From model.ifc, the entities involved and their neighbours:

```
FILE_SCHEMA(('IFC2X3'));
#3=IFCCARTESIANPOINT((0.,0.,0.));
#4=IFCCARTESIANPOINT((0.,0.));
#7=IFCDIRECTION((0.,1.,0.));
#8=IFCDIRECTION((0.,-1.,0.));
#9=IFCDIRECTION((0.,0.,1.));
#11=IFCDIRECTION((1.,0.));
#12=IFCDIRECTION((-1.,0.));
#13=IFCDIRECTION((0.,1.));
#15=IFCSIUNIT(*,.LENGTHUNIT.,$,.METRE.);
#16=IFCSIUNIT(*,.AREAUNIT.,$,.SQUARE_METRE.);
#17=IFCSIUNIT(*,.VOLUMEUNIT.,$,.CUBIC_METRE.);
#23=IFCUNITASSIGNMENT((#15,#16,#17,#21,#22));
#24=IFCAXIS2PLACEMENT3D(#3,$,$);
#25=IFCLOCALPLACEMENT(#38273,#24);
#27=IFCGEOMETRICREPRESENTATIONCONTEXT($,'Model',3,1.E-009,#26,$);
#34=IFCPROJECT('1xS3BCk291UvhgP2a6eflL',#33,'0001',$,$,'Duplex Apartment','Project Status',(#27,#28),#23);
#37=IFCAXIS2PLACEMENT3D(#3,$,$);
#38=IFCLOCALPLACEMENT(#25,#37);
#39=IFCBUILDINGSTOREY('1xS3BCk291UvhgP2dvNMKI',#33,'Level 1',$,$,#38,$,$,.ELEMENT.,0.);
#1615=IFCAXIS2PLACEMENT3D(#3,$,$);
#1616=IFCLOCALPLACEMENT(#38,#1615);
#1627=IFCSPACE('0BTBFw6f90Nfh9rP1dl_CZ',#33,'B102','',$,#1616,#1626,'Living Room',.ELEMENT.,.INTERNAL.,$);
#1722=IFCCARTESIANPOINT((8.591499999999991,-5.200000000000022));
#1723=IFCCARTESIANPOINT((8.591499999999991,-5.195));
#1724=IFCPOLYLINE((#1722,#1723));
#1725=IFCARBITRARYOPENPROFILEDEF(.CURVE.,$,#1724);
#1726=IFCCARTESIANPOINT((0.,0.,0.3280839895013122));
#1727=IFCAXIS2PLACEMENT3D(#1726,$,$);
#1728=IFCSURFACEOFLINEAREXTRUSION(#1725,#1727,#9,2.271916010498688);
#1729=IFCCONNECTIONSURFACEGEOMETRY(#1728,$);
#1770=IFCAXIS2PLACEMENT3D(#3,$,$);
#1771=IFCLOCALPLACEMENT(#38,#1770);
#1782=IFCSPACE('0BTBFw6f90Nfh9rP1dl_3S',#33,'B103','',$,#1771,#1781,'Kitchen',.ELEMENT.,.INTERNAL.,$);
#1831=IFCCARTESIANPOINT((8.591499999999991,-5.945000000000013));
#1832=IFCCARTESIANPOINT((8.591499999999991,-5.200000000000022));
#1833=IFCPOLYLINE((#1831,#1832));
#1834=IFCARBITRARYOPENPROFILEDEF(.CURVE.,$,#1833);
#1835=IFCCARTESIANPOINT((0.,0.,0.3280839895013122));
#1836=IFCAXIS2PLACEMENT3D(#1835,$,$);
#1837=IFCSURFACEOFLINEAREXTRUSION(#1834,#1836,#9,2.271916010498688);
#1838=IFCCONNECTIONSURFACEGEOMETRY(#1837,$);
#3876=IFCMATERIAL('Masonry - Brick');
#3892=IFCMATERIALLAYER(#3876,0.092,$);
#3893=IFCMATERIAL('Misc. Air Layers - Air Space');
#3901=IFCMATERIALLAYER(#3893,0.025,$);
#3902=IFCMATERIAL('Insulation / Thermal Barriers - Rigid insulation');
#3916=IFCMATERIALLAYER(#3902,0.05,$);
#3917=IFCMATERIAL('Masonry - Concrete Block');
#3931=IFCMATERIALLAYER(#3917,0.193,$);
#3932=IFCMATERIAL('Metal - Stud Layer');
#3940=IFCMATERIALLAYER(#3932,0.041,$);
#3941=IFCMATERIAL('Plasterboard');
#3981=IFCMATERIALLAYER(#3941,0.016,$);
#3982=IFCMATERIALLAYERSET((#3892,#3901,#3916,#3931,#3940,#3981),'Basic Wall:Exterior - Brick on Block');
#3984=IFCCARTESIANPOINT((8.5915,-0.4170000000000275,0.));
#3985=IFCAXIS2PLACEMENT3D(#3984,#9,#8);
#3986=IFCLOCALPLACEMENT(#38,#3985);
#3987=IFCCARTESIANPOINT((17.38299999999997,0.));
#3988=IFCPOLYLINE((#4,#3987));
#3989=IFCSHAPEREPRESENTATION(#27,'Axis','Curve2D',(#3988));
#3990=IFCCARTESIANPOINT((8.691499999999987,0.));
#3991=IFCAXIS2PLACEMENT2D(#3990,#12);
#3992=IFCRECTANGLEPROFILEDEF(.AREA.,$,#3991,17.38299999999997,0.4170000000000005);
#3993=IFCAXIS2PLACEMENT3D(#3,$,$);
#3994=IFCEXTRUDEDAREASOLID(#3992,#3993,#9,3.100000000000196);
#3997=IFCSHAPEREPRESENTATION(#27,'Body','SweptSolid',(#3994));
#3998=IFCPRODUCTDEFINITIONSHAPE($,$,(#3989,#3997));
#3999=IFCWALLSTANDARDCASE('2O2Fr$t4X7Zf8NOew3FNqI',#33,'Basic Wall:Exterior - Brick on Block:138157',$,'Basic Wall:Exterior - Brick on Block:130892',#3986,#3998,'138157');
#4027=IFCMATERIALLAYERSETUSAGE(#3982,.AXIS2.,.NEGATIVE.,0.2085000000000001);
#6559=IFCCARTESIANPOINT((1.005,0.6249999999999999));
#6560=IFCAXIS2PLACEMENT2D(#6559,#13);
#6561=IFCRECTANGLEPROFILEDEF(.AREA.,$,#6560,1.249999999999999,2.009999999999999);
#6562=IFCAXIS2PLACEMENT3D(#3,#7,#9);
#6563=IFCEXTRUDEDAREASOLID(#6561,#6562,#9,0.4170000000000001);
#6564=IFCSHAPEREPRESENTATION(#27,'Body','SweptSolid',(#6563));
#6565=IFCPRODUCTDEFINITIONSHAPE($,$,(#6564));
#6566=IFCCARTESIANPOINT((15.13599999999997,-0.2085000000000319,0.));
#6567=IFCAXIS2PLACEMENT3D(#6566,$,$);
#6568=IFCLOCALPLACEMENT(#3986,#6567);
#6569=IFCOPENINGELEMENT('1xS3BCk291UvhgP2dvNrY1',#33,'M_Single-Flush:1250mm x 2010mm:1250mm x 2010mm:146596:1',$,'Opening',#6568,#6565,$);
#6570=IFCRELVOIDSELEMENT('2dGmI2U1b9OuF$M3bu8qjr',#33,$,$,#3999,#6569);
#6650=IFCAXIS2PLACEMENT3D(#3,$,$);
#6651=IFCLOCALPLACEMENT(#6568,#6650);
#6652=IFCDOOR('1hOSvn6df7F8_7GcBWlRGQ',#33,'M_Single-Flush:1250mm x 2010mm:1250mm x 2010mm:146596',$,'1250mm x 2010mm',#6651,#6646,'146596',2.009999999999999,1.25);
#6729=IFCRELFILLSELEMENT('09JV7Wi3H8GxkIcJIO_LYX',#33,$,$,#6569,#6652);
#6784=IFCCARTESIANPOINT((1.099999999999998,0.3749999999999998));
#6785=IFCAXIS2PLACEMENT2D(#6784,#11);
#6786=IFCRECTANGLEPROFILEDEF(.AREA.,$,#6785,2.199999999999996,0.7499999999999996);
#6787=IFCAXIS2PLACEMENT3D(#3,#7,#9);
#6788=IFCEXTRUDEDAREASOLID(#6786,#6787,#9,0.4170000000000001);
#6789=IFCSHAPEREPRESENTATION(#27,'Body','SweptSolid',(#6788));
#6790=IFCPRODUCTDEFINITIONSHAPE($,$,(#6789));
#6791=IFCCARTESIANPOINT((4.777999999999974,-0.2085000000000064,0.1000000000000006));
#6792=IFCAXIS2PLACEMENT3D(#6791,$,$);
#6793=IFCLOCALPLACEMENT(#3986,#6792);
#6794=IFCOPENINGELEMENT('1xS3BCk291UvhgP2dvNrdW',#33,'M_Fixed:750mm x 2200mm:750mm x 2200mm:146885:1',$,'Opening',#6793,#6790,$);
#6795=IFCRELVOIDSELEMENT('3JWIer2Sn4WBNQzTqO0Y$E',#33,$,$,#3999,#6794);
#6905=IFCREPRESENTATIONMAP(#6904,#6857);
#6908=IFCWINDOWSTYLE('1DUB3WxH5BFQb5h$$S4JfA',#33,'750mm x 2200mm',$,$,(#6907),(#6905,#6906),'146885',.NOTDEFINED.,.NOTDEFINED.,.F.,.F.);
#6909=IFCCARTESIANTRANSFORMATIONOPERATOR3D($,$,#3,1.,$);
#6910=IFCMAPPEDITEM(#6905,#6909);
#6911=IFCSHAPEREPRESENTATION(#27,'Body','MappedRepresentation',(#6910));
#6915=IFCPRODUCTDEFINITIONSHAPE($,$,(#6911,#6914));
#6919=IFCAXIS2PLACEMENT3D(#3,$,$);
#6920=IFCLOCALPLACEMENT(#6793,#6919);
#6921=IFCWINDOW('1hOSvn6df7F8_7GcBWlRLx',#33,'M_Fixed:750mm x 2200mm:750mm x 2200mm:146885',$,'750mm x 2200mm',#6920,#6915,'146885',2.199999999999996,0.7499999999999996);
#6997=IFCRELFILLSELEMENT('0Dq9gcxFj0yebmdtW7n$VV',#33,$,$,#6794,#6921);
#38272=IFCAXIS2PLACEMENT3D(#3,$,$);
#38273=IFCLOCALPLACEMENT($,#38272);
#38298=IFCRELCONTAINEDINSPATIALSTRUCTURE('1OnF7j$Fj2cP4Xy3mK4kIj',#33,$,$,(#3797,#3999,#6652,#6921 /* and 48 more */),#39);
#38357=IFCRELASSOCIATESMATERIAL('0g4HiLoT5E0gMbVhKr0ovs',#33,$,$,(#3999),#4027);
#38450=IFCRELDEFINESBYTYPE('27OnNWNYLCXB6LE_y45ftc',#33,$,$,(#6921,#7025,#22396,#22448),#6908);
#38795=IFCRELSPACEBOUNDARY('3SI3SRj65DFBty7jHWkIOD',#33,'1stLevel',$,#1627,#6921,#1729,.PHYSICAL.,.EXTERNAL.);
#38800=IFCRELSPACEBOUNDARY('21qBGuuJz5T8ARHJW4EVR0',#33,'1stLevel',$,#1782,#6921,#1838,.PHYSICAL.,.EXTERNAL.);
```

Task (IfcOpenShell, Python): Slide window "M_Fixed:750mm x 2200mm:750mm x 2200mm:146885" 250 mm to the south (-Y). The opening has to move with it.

```python
import numpy as np
import ifcopenshell
import ifcopenshell.api.geometry
import ifcopenshell.util.placement
import ifcopenshell.util.unit

model = ifcopenshell.open("model.ifc")
unit_scale = ifcopenshell.util.unit.calculate_unit_scale(model)

window = model.by_id(6921)
opening = window.FillsVoids[0].RelatingOpeningElement
wall = opening.VoidsElements[0].RelatingBuildingElement

wall_matrix = ifcopenshell.util.placement.get_local_placement(wall.ObjectPlacement)
shift = wall_matrix[:3, 0] * 0.25 / unit_scale
before = ifcopenshell.util.placement.get_local_placement(window.ObjectPlacement)[:3, 3].copy()

# The window is placed relative to its opening, so it follows when the opening moves.
matrix = ifcopenshell.util.placement.get_local_placement(opening.ObjectPlacement)
matrix[:3, 3] += shift
ifcopenshell.api.geometry.edit_object_placement(
    model, product=opening, matrix=matrix, is_si=False, should_transform_children=True
)

# Space boundary surfaces are stored in each space's coordinates; move them too.
for rel in window.ProvidesBoundaries:
    if not rel.ConnectionGeometry:
        continue
    surface = rel.ConnectionGeometry.SurfaceOnRelatingElement
    space_matrix = ifcopenshell.util.placement.get_local_placement(rel.RelatingSpace.ObjectPlacement)
    point = np.array(surface.Position.Location.Coordinates) + space_matrix[:3, :3].T @ shift
    surface.Position = model.createIfcAxis2Placement3D(
        model.createIfcCartesianPoint(point.tolist()), surface.Position.Axis, surface.Position.RefDirection
    )

after = ifcopenshell.util.placement.get_local_placement(window.ObjectPlacement)[:3, 3]
print("window moved by", (after - before).round(3) + 0.0)

model.write("model_updated.ifc")
```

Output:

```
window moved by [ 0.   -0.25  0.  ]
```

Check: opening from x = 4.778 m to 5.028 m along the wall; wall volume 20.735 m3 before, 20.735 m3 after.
